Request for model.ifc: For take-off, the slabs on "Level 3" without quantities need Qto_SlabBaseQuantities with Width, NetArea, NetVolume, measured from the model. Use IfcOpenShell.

First a look at what the model holds.

```python
import ifcopenshell
import ifcopenshell.util.element
import ifcopenshell.util.unit

model = ifcopenshell.open("model.ifc")
print(model.schema)
for unit_type in ("LENGTHUNIT", "AREAUNIT", "VOLUMEUNIT"):
    print(unit_type, ifcopenshell.util.unit.calculate_unit_scale(model, unit_type))
storey = next(s for s in model.by_type("IfcBuildingStorey") if s.Name == "Level 3")
slabs = [e for e in ifcopenshell.util.element.get_decomposition(storey) if e.is_a("IfcSlab")]
for e in sorted(slabs, key=lambda e: e.id()):
    print(e.id(), e.is_a(), e.Name, list(ifcopenshell.util.element.get_psets(e, qtos_only=True)), sep=" | ")
```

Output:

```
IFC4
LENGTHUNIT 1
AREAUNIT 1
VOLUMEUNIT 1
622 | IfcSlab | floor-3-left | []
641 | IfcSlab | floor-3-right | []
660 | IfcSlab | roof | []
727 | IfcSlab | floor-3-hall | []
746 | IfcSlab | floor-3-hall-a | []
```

```python
import ifcopenshell
import ifcopenshell.api.pset
import ifcopenshell.geom
import ifcopenshell.util.element
import ifcopenshell.util.shape
import ifcopenshell.util.unit

model = ifcopenshell.open("model.ifc")
unit_scale = ifcopenshell.util.unit.calculate_unit_scale(model)
area_scale = ifcopenshell.util.unit.calculate_unit_scale(model, "AREAUNIT")
volume_scale = ifcopenshell.util.unit.calculate_unit_scale(model, "VOLUMEUNIT")
settings = ifcopenshell.geom.settings()

storey = next(s for s in model.by_type("IfcBuildingStorey") if s.Name == "Level 3")
slabs = [e for e in ifcopenshell.util.element.get_decomposition(storey) if e.is_a("IfcSlab")]

for e in sorted(slabs, key=lambda e: e.id()):
    if ifcopenshell.util.element.get_psets(e, qtos_only=True, should_inherit=False):
        continue
    # Geometry comes back in metres, in the element's own axes.
    shape = ifcopenshell.geom.create_shape(settings, e)
    values = {
        "Width": ifcopenshell.util.shape.get_z(shape.geometry) / unit_scale,
        "NetArea": ifcopenshell.util.shape.get_footprint_area(shape.geometry) / area_scale,
        "NetVolume": ifcopenshell.util.shape.get_volume(shape.geometry) / volume_scale,
    }
    qto = ifcopenshell.api.pset.add_qto(model, product=e, name="Qto_SlabBaseQuantities")
    ifcopenshell.api.pset.edit_qto(model, qto=qto, properties=values)
    print(e.id(), {k: round(v, 3) for k, v in values.items()})

model.write("model-out.ifc")
```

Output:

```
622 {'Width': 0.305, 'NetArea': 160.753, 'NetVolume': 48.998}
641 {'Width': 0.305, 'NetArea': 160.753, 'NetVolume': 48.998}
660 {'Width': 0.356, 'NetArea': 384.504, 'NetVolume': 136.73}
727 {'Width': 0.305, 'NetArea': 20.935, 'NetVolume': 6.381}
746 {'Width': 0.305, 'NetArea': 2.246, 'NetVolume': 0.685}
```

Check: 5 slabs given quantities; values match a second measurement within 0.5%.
